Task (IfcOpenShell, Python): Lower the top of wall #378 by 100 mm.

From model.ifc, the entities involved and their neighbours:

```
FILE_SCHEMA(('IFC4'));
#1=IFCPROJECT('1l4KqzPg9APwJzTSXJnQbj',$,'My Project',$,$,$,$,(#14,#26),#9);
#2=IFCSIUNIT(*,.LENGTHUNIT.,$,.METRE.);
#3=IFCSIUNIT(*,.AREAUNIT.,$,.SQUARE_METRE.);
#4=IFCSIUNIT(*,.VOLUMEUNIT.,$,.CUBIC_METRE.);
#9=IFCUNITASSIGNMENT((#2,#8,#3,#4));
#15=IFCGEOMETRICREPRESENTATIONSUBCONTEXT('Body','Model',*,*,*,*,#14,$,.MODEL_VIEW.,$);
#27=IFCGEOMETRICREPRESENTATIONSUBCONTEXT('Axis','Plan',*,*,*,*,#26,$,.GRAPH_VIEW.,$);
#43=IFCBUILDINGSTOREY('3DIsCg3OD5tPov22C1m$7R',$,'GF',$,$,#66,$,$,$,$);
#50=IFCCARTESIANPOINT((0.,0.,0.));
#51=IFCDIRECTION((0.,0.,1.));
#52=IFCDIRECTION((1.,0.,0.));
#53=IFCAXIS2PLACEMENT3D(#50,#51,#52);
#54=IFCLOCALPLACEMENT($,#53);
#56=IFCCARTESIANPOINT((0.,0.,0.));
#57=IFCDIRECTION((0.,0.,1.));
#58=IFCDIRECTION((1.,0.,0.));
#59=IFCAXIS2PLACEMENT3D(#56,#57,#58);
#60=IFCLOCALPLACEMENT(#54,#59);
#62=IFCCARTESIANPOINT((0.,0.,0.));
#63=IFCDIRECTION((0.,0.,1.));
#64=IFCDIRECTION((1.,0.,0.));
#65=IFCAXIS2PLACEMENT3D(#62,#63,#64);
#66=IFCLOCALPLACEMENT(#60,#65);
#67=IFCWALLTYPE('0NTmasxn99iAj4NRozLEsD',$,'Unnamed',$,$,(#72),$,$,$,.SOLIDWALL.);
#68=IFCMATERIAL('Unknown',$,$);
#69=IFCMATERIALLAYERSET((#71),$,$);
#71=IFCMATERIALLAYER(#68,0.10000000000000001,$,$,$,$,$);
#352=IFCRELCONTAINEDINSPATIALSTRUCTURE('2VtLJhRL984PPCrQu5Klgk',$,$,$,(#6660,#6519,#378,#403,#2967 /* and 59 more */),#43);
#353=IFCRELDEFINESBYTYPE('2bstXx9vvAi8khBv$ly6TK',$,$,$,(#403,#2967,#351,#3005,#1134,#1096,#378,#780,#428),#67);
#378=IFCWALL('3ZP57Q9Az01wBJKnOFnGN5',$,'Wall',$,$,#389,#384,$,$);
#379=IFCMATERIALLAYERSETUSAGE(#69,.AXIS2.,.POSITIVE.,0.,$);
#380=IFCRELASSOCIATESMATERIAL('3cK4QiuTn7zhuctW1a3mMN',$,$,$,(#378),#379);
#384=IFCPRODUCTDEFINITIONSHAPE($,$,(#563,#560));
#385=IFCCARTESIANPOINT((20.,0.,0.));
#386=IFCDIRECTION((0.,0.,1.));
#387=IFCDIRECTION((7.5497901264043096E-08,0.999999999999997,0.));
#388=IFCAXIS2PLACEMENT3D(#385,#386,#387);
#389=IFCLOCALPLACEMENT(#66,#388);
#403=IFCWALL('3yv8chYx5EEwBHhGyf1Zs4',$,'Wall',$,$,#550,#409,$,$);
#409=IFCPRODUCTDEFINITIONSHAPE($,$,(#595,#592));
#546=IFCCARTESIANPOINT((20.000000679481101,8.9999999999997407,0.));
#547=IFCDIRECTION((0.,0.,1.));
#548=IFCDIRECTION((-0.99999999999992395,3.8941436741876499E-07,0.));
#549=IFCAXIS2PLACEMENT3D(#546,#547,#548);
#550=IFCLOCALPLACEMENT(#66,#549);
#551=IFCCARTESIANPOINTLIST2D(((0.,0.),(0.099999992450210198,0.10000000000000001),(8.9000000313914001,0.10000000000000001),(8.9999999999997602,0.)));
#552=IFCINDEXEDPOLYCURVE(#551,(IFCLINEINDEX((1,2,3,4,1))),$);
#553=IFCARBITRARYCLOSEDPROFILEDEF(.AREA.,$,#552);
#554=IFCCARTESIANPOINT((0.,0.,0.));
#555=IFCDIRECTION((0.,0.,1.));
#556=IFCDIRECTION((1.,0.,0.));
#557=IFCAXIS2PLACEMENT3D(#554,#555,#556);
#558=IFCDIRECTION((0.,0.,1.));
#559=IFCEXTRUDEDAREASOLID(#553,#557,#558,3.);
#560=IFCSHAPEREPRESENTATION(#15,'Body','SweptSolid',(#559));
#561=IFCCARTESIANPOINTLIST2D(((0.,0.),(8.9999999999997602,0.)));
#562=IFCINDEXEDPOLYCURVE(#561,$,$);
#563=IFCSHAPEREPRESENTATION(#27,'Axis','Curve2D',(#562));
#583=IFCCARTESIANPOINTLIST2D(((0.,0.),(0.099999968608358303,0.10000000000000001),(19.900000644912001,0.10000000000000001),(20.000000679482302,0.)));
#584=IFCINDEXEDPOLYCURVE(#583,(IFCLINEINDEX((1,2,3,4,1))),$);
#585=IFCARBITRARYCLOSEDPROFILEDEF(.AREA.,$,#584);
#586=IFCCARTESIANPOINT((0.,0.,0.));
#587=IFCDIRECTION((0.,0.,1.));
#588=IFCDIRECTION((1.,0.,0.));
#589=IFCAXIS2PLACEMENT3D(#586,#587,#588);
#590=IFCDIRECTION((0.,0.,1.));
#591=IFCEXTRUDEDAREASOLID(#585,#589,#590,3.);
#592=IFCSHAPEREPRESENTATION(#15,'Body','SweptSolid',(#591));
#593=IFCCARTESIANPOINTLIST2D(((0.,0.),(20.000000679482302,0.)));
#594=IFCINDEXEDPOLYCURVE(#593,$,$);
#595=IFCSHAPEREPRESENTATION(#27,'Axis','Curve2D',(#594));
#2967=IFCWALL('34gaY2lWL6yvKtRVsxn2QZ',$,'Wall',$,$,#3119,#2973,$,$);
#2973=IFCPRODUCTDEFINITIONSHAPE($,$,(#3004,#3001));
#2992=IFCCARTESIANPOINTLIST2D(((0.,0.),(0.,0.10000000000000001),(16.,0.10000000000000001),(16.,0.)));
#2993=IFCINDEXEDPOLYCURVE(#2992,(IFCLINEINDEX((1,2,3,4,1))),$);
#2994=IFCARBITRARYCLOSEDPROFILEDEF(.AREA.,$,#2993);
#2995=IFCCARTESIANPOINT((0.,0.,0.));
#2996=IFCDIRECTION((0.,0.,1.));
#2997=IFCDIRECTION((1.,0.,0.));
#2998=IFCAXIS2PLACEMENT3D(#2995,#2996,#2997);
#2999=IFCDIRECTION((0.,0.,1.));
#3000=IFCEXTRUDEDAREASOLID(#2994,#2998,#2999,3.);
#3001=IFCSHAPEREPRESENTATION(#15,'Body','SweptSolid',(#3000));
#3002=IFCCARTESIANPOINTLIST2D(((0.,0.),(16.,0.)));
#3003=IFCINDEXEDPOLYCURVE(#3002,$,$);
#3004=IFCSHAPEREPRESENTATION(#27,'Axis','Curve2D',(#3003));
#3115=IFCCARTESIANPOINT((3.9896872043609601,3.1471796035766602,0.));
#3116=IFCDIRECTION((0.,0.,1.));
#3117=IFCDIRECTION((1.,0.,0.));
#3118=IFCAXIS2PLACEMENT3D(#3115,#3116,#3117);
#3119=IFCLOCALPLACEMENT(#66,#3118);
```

```python
import ifcopenshell
import ifcopenshell.geom
import ifcopenshell.util.representation
import ifcopenshell.util.shape

model = ifcopenshell.open("model.ifc")
settings = ifcopenshell.geom.settings()


def volume(element):
    """Net volume in cubic metres, openings subtracted."""
    shape = ifcopenshell.geom.create_shape(settings, element)
    return ifcopenshell.util.shape.get_volume(shape.geometry)


wall = model.by_guid("3ZP57Q9Az01wBJKnOFnGN5")
before = volume(wall)

body = ifcopenshell.util.representation.get_representation(wall, "Model", "Body")
solid = body.Items[0]
old_height = solid.Depth
solid.Depth -= 0.1
after = volume(wall)

print(f"height {old_height:g} -> {solid.Depth:g}, volume {before:.3f} -> {after:.3f} m3")

model.write("model_v2.ifc")
```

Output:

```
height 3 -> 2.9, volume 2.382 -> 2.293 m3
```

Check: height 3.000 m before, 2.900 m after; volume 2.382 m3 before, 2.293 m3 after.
